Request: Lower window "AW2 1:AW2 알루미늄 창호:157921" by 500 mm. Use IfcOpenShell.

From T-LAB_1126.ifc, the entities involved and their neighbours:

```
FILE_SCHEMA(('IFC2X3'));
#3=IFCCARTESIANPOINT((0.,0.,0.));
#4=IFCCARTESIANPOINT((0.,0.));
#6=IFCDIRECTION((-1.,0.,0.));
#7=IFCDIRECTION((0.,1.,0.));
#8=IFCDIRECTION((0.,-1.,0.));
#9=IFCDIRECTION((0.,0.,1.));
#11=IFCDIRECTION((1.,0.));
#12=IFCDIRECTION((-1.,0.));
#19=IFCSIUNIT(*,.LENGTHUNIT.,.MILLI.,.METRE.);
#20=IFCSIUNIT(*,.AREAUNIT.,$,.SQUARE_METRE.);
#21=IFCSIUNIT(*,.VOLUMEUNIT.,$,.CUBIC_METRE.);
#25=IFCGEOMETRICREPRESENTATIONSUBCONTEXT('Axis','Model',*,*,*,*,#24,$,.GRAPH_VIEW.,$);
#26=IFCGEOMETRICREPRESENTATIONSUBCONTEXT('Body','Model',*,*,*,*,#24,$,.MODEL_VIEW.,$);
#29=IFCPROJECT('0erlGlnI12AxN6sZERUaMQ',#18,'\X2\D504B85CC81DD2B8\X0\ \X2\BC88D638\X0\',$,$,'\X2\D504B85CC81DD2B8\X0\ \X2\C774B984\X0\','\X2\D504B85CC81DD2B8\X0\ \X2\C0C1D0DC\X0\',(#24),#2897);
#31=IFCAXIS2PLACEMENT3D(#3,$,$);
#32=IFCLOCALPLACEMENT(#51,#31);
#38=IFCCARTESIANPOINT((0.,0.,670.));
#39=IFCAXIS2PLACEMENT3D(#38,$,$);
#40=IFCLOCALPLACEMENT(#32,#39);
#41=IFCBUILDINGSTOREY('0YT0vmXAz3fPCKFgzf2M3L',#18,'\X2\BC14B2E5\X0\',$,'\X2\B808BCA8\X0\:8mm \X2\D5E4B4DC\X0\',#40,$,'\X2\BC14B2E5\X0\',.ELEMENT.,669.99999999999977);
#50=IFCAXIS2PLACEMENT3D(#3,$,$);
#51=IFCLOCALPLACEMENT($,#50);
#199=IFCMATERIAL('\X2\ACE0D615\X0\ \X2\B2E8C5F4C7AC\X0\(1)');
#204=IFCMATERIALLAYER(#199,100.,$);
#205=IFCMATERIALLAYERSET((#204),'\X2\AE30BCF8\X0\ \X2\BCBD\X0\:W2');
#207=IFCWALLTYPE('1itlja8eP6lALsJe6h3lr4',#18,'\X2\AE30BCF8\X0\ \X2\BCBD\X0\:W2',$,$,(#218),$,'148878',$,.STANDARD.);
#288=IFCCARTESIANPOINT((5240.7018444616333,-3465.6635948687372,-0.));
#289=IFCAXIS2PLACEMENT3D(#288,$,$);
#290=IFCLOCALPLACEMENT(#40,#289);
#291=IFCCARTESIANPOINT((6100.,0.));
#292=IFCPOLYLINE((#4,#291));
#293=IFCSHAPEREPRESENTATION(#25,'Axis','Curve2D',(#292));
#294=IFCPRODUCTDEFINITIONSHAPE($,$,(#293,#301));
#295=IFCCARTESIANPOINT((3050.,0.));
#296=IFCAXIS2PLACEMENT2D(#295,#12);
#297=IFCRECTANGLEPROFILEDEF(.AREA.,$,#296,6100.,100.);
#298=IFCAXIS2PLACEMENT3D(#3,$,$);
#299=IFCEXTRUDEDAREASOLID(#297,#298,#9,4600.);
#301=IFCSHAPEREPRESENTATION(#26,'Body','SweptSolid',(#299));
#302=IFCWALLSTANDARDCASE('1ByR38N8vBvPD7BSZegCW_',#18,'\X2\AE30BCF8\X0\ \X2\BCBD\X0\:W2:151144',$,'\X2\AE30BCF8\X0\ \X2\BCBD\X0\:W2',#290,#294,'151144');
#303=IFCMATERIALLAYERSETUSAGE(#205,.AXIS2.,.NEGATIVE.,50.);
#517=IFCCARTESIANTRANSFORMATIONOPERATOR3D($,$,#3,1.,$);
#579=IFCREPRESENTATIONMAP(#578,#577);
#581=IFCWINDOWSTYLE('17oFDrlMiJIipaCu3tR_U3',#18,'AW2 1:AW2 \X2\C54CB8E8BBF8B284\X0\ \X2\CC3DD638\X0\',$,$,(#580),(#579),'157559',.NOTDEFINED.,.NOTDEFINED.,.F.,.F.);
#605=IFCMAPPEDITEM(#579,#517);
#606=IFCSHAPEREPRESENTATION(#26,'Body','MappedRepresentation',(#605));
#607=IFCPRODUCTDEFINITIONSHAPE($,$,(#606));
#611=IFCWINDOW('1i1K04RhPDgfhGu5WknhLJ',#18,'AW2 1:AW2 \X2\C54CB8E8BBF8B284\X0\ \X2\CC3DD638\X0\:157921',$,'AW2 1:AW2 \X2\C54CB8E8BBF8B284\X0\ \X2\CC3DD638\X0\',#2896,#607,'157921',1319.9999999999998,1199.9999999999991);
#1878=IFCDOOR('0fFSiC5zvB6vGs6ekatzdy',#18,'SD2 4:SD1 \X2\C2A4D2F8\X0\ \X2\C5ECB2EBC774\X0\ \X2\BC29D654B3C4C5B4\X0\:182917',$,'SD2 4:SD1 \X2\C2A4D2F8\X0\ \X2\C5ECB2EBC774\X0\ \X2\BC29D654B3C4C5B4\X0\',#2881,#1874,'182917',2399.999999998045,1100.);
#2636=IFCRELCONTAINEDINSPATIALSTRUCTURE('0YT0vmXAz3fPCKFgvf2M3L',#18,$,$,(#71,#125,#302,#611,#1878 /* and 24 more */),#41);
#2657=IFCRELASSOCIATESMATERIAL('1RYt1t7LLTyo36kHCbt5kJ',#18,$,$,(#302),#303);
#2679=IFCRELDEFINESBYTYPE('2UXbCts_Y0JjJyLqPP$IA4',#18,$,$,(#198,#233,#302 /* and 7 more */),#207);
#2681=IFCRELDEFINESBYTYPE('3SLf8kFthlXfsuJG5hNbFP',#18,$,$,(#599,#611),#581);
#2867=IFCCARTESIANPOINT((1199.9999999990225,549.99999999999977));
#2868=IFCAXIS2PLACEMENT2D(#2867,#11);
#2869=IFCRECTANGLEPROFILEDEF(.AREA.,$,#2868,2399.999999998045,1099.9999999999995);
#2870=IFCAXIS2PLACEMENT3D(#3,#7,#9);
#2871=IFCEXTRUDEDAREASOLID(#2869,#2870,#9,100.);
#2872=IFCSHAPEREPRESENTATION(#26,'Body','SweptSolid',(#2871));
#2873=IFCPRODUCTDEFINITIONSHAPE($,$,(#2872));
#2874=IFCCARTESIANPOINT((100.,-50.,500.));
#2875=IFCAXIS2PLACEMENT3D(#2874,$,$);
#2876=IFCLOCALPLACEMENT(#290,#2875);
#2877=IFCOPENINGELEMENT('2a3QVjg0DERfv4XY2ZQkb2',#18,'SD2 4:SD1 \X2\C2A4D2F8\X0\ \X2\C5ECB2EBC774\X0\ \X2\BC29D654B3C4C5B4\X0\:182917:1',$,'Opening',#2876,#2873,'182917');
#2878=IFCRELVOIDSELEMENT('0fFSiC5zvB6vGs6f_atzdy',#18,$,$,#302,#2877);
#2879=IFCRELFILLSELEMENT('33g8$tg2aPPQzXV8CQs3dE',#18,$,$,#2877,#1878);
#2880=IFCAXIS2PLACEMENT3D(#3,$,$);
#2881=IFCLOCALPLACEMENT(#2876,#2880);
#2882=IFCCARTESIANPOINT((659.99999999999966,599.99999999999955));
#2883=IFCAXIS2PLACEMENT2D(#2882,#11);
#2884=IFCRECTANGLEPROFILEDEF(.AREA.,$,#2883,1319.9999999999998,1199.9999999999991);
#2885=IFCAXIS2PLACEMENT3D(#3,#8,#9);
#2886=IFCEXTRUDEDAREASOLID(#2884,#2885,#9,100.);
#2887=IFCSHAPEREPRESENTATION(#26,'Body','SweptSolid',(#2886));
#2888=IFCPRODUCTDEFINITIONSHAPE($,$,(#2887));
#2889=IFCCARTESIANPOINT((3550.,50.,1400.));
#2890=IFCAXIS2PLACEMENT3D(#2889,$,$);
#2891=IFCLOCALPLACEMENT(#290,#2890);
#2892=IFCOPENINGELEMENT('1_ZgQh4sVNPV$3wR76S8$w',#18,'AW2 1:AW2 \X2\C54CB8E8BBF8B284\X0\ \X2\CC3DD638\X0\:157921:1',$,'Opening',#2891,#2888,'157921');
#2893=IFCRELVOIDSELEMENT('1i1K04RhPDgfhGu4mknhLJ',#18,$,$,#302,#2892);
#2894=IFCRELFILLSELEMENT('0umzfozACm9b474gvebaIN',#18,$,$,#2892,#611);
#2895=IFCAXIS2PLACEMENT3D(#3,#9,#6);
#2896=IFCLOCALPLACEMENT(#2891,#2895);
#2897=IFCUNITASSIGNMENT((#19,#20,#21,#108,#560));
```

```python
import numpy as np
import ifcopenshell
import ifcopenshell.api.geometry
import ifcopenshell.util.placement
import ifcopenshell.util.unit

model = ifcopenshell.open("T-LAB_1126.ifc")
unit_scale = ifcopenshell.util.unit.calculate_unit_scale(model)

window = model.by_guid("1i1K04RhPDgfhGu5WknhLJ")
opening = window.FillsVoids[0].RelatingOpeningElement
dz = -0.5 / unit_scale

shift = np.array([0.0, 0.0, dz])
# The window is placed relative to its opening, so it follows when the opening moves.
matrix = ifcopenshell.util.placement.get_local_placement(opening.ObjectPlacement)
matrix[:3, 3] += shift
ifcopenshell.api.geometry.edit_object_placement(
    model, product=opening, matrix=matrix, is_si=False, should_transform_children=True
)

print(f"moved by {dz * unit_scale:+.3f} m")

model.write("T-LAB_1126_updated.ifc")
```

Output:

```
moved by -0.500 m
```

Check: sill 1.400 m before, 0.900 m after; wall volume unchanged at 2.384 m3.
